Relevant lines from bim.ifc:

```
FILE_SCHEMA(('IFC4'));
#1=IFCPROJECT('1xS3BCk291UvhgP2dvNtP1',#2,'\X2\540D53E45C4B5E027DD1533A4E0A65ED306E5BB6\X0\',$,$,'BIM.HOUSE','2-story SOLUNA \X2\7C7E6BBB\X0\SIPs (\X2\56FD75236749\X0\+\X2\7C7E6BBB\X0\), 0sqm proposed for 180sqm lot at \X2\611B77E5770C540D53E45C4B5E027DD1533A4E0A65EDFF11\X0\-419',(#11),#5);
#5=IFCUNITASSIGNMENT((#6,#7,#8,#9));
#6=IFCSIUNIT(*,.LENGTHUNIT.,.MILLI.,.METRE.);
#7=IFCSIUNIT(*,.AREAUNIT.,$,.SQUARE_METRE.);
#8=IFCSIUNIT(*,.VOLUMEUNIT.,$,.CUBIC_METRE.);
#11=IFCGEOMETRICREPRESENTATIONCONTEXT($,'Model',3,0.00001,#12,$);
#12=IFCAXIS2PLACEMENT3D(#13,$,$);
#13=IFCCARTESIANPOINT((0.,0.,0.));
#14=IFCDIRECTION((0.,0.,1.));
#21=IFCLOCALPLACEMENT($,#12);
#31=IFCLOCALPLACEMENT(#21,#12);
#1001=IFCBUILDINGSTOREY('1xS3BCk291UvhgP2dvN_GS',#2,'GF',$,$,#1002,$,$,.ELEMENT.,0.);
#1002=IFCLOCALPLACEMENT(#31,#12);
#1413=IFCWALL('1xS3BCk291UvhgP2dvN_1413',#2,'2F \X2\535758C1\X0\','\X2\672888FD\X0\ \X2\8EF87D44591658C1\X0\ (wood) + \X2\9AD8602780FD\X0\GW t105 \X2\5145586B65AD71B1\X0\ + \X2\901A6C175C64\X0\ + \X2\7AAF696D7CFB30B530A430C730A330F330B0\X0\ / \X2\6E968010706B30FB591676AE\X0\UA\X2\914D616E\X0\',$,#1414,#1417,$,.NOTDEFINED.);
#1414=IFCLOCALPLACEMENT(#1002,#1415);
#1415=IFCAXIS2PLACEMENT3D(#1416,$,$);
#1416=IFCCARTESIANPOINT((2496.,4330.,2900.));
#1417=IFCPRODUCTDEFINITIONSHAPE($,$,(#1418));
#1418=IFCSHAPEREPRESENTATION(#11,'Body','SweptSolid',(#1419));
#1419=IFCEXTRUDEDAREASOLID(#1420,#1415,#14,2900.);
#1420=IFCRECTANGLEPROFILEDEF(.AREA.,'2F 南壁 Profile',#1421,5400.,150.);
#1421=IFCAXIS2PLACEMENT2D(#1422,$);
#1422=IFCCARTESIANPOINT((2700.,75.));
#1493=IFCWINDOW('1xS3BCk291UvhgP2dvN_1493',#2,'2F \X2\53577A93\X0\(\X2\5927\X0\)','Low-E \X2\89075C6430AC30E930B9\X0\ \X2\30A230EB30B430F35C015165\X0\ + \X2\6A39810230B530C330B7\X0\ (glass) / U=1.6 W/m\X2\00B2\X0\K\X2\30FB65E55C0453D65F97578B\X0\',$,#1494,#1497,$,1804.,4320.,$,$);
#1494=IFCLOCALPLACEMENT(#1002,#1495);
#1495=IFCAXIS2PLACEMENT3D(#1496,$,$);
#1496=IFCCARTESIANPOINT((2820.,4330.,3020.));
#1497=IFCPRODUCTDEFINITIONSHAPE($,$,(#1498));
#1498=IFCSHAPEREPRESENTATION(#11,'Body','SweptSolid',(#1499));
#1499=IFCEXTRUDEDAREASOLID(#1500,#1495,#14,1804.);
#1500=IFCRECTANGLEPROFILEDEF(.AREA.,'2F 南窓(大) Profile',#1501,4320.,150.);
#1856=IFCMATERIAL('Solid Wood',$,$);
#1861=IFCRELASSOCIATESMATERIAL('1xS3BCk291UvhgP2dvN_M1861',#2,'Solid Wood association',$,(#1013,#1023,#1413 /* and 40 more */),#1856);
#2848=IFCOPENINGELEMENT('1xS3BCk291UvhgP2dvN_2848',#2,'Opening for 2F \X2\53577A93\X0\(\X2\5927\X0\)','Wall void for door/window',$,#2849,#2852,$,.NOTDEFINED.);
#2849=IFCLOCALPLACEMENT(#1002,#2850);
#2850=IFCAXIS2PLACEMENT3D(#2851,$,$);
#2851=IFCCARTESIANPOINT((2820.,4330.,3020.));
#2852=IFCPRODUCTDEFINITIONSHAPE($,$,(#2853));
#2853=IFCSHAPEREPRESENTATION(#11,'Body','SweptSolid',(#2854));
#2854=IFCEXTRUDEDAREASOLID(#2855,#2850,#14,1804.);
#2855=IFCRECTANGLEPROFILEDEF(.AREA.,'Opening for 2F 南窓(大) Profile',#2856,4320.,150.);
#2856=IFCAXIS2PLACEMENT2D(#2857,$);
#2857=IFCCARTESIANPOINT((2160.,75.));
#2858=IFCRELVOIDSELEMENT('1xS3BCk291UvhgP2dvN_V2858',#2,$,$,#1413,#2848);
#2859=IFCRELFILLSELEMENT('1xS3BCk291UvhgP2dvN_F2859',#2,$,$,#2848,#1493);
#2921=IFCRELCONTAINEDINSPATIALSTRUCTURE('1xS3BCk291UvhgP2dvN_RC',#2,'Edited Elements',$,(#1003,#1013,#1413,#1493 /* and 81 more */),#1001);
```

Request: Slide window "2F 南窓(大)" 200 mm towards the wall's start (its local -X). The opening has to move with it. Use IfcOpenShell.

```python
import ifcopenshell
import ifcopenshell.api.geometry
import ifcopenshell.util.placement
import ifcopenshell.util.unit

model = ifcopenshell.open("bim.ifc")
unit_scale = ifcopenshell.util.unit.calculate_unit_scale(model)

window = model.by_guid("1xS3BCk291UvhgP2dvN_1493")
opening = window.FillsVoids[0].RelatingOpeningElement
wall = opening.VoidsElements[0].RelatingBuildingElement

wall_matrix = ifcopenshell.util.placement.get_local_placement(wall.ObjectPlacement)
shift = wall_matrix[:3, 0] * -0.2 / unit_scale
before = ifcopenshell.util.placement.get_local_placement(window.ObjectPlacement)[:3, 3].copy()

# The window is not placed relative to its opening, so move both.
for product in (opening, window):
    matrix = ifcopenshell.util.placement.get_local_placement(product.ObjectPlacement)
    matrix[:3, 3] += shift
    ifcopenshell.api.geometry.edit_object_placement(model, product=product, matrix=matrix, is_si=False)

after = ifcopenshell.util.placement.get_local_placement(window.ObjectPlacement)[:3, 3]
print("window moved by", (after - before).round(3) + 0.0)

model.write("bim_edited.ifc")
```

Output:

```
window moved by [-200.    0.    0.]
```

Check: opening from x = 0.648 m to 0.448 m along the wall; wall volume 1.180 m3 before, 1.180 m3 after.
